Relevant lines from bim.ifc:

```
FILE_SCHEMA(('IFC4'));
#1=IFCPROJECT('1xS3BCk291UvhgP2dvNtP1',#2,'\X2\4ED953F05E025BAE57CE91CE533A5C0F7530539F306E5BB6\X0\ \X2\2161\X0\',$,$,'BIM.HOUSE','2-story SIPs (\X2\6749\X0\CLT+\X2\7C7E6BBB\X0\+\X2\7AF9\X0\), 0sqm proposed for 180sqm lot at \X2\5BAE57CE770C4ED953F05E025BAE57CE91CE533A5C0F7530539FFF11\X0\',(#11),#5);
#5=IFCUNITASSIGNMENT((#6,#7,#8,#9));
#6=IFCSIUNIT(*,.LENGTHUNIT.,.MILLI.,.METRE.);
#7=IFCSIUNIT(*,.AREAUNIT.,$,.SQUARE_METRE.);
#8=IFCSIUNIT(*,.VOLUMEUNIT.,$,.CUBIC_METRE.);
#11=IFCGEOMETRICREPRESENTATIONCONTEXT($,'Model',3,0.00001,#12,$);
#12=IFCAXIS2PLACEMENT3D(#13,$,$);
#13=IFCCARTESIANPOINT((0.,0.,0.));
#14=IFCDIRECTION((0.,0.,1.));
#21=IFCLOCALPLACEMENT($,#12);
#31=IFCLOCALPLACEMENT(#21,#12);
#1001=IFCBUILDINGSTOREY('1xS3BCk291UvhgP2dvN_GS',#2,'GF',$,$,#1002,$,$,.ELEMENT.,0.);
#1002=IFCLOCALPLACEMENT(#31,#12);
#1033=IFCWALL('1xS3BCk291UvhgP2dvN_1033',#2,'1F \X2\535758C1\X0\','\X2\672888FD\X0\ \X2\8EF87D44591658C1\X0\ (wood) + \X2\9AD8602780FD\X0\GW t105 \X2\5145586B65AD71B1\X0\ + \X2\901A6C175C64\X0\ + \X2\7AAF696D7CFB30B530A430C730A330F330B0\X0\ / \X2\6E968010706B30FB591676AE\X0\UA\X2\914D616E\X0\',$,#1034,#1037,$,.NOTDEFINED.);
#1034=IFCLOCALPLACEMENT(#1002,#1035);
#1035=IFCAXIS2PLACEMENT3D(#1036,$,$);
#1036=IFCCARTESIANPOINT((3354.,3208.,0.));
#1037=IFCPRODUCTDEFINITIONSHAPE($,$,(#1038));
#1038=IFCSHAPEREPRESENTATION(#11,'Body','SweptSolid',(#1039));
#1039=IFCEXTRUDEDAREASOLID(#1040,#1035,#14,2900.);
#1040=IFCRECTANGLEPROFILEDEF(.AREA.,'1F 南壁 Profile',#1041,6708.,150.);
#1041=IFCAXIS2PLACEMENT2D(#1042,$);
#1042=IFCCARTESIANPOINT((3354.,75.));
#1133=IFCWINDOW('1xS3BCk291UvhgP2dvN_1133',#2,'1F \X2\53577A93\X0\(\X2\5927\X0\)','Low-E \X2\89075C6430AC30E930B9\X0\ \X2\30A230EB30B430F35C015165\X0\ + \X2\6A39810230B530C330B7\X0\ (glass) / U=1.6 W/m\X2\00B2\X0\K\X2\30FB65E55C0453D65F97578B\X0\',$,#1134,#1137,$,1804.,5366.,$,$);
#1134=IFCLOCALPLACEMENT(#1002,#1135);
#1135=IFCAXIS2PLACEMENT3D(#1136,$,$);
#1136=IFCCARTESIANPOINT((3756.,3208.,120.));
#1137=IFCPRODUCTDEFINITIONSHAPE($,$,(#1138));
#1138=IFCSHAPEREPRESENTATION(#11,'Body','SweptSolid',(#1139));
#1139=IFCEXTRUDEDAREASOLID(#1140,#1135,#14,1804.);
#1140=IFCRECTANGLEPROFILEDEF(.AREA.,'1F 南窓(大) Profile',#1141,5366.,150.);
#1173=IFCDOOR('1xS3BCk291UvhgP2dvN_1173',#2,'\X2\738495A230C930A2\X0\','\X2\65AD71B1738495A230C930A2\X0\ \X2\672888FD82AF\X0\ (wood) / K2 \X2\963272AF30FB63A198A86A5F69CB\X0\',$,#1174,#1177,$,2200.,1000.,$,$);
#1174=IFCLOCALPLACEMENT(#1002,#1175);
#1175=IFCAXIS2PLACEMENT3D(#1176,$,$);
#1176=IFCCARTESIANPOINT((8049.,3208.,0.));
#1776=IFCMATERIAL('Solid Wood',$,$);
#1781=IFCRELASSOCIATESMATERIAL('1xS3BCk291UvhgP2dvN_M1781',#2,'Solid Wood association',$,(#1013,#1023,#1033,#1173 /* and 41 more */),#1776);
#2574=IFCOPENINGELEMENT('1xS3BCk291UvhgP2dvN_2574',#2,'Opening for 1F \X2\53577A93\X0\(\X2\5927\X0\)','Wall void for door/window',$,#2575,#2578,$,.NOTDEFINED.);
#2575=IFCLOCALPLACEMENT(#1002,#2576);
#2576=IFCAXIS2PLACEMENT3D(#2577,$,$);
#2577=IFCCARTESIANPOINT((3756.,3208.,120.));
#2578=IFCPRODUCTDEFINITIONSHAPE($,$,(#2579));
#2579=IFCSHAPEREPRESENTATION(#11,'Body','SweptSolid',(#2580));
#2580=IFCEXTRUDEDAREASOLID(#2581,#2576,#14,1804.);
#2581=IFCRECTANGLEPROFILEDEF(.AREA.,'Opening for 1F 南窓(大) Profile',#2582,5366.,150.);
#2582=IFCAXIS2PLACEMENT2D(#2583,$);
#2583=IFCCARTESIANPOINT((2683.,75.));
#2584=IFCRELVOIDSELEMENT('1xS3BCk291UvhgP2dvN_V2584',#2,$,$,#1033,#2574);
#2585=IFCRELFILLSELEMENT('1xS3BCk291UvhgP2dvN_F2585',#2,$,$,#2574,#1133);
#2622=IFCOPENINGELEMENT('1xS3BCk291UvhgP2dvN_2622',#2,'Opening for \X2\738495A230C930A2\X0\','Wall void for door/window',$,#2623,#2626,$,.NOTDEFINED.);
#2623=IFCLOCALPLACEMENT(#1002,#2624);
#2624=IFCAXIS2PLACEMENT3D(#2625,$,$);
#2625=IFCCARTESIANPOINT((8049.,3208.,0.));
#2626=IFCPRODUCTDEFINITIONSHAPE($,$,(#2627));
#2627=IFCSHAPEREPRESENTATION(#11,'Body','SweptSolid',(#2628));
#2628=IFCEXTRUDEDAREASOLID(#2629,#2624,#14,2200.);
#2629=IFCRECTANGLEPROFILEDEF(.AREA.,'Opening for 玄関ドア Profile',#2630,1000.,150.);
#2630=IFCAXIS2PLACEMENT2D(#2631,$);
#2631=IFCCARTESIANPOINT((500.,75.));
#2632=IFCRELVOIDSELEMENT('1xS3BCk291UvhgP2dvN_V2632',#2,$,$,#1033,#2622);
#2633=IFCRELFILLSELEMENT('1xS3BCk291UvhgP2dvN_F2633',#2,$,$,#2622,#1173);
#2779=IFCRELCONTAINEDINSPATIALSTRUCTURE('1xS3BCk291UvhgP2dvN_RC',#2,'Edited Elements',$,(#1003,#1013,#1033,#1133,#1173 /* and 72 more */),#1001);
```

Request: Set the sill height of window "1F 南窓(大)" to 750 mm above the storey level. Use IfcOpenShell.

```python
import numpy as np
import ifcopenshell
import ifcopenshell.api.geometry
import ifcopenshell.geom
import ifcopenshell.util.element
import ifcopenshell.util.placement
import ifcopenshell.util.shape
import ifcopenshell.util.unit

model = ifcopenshell.open("bim.ifc")
unit_scale = ifcopenshell.util.unit.calculate_unit_scale(model)

window = model.by_id(1133)
opening = window.FillsVoids[0].RelatingOpeningElement
storey = ifcopenshell.util.element.get_container(window, ifc_class="IfcBuildingStorey")
level = ifcopenshell.util.placement.get_local_placement(storey.ObjectPlacement)[2, 3]

# The opening's origin need not be at the sill, so measure its lowest point.
shape = ifcopenshell.geom.create_shape(ifcopenshell.geom.settings(), opening)
bottom = ifcopenshell.util.shape.get_shape_bottom_elevation(shape, shape.geometry) / unit_scale
dz = level + 750.0 - bottom

shift = np.array([0.0, 0.0, dz])
# The window is not placed relative to its opening, so move both.
for product in (opening, window):
    matrix = ifcopenshell.util.placement.get_local_placement(product.ObjectPlacement)
    matrix[:3, 3] += shift
    ifcopenshell.api.geometry.edit_object_placement(model, product=product, matrix=matrix, is_si=False)

print(f"moved by {dz * unit_scale:+.3f} m")

model.write("bim-out.ifc")
```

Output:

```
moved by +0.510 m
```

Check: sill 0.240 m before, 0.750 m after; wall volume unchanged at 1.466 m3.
